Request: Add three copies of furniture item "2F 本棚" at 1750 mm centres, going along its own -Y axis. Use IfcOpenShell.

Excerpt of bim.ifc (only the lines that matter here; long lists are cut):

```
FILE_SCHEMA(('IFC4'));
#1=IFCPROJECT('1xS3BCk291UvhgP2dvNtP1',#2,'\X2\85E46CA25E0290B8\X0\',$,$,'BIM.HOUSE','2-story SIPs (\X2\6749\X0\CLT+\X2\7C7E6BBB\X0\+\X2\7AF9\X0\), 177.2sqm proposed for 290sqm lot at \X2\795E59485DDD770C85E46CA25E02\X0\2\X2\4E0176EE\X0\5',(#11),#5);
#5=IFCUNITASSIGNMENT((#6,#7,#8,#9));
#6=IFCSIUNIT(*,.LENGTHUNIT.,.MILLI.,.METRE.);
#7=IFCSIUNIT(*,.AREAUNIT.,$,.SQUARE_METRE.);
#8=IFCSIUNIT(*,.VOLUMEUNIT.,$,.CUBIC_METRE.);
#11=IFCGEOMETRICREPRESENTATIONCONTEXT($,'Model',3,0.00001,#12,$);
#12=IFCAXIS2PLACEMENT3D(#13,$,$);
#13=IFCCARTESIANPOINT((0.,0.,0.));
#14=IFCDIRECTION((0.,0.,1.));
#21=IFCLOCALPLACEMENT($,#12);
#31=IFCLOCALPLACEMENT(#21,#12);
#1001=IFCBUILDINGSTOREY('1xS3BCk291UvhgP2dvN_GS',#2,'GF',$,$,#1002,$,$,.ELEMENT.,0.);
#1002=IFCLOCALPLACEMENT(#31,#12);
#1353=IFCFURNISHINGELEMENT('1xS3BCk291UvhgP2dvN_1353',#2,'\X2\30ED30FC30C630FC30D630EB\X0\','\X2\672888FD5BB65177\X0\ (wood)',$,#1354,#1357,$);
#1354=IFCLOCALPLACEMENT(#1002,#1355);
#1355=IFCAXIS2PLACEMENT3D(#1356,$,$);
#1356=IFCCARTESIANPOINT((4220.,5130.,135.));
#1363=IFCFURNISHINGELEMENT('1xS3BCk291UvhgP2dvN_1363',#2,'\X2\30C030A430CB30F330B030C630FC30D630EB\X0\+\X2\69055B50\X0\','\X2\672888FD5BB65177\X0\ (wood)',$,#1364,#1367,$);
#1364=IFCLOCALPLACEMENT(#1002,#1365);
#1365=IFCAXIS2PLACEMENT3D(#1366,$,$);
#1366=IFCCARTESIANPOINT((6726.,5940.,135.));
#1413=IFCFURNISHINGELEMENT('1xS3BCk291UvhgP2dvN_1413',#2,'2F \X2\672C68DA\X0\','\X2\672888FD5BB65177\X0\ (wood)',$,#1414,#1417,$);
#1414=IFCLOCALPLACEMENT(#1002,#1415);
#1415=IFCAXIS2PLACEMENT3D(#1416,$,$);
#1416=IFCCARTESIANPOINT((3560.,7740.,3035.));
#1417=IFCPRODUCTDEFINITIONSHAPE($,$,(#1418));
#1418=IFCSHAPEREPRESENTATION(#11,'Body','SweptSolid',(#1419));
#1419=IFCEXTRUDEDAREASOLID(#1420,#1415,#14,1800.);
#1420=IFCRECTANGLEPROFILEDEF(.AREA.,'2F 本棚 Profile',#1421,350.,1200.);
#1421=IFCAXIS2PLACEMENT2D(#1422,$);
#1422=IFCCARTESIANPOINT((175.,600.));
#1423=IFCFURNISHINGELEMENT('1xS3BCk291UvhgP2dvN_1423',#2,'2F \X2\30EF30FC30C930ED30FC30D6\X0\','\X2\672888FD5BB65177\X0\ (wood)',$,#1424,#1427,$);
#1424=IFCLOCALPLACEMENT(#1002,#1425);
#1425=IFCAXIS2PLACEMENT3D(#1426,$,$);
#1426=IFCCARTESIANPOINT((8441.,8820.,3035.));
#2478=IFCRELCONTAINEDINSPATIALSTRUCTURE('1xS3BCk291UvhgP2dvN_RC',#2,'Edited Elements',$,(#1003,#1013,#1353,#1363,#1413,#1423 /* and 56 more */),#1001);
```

```python
import ifcopenshell
import ifcopenshell.api.geometry
import ifcopenshell.api.root
import ifcopenshell.util.element
import ifcopenshell.util.placement
import ifcopenshell.util.unit

model = ifcopenshell.open("bim.ifc")
unit_scale = ifcopenshell.util.unit.calculate_unit_scale(model)


def reuse_history(source, copy):
    """copy_class also copies each property set's owner history, people and application; keep the originals."""
    for rel in copy.IsDefinedBy:
        if rel.is_a("IfcRelDefinesByProperties") and (history := rel.RelatingPropertyDefinition.OwnerHistory):
            rel.RelatingPropertyDefinition.OwnerHistory = source.OwnerHistory
            ifcopenshell.util.element.remove_deep2(model, history)


source = model.by_guid("1xS3BCk291UvhgP2dvN_1413")
base = ifcopenshell.util.placement.get_local_placement(source.ObjectPlacement)
step = -base[:3, 1] * 1.75 / unit_scale

for i in range(1, 4):
    copy = ifcopenshell.api.root.copy_class(model, product=source)
    copy.Representation = ifcopenshell.util.element.copy_deep(
        model, source.Representation, exclude=["IfcGeometricRepresentationContext", "IfcRepresentationMap"]
    )
    reuse_history(source, copy)
    matrix = base.copy()
    matrix[:3, 3] += i * step
    print("added at", matrix[:3, 3].round(3) + 0.0)
    ifcopenshell.api.geometry.edit_object_placement(model, product=copy, matrix=matrix, is_si=False)

model.write("bim_updated.ifc")
```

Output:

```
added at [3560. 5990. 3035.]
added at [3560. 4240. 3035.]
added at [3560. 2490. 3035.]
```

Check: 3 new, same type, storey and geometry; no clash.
